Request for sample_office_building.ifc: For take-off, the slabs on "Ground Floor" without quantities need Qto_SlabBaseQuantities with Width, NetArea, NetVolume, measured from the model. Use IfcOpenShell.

First a look at what the model holds.

```python
import ifcopenshell
import ifcopenshell.util.element
import ifcopenshell.util.unit

model = ifcopenshell.open("sample_office_building.ifc")
print(model.schema)
for unit_type in ("LENGTHUNIT", "AREAUNIT", "VOLUMEUNIT"):
    print(unit_type, ifcopenshell.util.unit.calculate_unit_scale(model, unit_type))
storey = next(s for s in model.by_type("IfcBuildingStorey") if s.Name == "Ground Floor")
slabs = [e for e in ifcopenshell.util.element.get_decomposition(storey) if e.is_a("IfcSlab")]
for e in sorted(slabs, key=lambda e: e.id()):
    print(e.id(), e.is_a(), e.Name, list(ifcopenshell.util.element.get_psets(e, qtos_only=True)), sep=" | ")
```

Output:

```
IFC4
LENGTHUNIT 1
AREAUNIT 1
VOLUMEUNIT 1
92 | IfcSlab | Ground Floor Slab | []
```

```python
import ifcopenshell
import ifcopenshell.api.pset
import ifcopenshell.geom
import ifcopenshell.util.element
import ifcopenshell.util.shape
import ifcopenshell.util.unit

model = ifcopenshell.open("sample_office_building.ifc")
unit_scale = ifcopenshell.util.unit.calculate_unit_scale(model)
area_scale = ifcopenshell.util.unit.calculate_unit_scale(model, "AREAUNIT")
volume_scale = ifcopenshell.util.unit.calculate_unit_scale(model, "VOLUMEUNIT")
settings = ifcopenshell.geom.settings()

storey = next(s for s in model.by_type("IfcBuildingStorey") if s.Name == "Ground Floor")
slabs = [e for e in ifcopenshell.util.element.get_decomposition(storey) if e.is_a("IfcSlab")]

for e in sorted(slabs, key=lambda e: e.id()):
    if ifcopenshell.util.element.get_psets(e, qtos_only=True, should_inherit=False):
        continue
    # Geometry comes back in metres, in the element's own axes.
    shape = ifcopenshell.geom.create_shape(settings, e)
    values = {
        "Width": ifcopenshell.util.shape.get_z(shape.geometry) / unit_scale,
        "NetArea": ifcopenshell.util.shape.get_footprint_area(shape.geometry) / area_scale,
        "NetVolume": ifcopenshell.util.shape.get_volume(shape.geometry) / volume_scale,
    }
    qto = ifcopenshell.api.pset.add_qto(model, product=e, name="Qto_SlabBaseQuantities")
    ifcopenshell.api.pset.edit_qto(model, qto=qto, properties=values)
    print(e.id(), {k: round(v, 3) for k, v in values.items()})

model.write("sample_office_building_edited.ifc")
```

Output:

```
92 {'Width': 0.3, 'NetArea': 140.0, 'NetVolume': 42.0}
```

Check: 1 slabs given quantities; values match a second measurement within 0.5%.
